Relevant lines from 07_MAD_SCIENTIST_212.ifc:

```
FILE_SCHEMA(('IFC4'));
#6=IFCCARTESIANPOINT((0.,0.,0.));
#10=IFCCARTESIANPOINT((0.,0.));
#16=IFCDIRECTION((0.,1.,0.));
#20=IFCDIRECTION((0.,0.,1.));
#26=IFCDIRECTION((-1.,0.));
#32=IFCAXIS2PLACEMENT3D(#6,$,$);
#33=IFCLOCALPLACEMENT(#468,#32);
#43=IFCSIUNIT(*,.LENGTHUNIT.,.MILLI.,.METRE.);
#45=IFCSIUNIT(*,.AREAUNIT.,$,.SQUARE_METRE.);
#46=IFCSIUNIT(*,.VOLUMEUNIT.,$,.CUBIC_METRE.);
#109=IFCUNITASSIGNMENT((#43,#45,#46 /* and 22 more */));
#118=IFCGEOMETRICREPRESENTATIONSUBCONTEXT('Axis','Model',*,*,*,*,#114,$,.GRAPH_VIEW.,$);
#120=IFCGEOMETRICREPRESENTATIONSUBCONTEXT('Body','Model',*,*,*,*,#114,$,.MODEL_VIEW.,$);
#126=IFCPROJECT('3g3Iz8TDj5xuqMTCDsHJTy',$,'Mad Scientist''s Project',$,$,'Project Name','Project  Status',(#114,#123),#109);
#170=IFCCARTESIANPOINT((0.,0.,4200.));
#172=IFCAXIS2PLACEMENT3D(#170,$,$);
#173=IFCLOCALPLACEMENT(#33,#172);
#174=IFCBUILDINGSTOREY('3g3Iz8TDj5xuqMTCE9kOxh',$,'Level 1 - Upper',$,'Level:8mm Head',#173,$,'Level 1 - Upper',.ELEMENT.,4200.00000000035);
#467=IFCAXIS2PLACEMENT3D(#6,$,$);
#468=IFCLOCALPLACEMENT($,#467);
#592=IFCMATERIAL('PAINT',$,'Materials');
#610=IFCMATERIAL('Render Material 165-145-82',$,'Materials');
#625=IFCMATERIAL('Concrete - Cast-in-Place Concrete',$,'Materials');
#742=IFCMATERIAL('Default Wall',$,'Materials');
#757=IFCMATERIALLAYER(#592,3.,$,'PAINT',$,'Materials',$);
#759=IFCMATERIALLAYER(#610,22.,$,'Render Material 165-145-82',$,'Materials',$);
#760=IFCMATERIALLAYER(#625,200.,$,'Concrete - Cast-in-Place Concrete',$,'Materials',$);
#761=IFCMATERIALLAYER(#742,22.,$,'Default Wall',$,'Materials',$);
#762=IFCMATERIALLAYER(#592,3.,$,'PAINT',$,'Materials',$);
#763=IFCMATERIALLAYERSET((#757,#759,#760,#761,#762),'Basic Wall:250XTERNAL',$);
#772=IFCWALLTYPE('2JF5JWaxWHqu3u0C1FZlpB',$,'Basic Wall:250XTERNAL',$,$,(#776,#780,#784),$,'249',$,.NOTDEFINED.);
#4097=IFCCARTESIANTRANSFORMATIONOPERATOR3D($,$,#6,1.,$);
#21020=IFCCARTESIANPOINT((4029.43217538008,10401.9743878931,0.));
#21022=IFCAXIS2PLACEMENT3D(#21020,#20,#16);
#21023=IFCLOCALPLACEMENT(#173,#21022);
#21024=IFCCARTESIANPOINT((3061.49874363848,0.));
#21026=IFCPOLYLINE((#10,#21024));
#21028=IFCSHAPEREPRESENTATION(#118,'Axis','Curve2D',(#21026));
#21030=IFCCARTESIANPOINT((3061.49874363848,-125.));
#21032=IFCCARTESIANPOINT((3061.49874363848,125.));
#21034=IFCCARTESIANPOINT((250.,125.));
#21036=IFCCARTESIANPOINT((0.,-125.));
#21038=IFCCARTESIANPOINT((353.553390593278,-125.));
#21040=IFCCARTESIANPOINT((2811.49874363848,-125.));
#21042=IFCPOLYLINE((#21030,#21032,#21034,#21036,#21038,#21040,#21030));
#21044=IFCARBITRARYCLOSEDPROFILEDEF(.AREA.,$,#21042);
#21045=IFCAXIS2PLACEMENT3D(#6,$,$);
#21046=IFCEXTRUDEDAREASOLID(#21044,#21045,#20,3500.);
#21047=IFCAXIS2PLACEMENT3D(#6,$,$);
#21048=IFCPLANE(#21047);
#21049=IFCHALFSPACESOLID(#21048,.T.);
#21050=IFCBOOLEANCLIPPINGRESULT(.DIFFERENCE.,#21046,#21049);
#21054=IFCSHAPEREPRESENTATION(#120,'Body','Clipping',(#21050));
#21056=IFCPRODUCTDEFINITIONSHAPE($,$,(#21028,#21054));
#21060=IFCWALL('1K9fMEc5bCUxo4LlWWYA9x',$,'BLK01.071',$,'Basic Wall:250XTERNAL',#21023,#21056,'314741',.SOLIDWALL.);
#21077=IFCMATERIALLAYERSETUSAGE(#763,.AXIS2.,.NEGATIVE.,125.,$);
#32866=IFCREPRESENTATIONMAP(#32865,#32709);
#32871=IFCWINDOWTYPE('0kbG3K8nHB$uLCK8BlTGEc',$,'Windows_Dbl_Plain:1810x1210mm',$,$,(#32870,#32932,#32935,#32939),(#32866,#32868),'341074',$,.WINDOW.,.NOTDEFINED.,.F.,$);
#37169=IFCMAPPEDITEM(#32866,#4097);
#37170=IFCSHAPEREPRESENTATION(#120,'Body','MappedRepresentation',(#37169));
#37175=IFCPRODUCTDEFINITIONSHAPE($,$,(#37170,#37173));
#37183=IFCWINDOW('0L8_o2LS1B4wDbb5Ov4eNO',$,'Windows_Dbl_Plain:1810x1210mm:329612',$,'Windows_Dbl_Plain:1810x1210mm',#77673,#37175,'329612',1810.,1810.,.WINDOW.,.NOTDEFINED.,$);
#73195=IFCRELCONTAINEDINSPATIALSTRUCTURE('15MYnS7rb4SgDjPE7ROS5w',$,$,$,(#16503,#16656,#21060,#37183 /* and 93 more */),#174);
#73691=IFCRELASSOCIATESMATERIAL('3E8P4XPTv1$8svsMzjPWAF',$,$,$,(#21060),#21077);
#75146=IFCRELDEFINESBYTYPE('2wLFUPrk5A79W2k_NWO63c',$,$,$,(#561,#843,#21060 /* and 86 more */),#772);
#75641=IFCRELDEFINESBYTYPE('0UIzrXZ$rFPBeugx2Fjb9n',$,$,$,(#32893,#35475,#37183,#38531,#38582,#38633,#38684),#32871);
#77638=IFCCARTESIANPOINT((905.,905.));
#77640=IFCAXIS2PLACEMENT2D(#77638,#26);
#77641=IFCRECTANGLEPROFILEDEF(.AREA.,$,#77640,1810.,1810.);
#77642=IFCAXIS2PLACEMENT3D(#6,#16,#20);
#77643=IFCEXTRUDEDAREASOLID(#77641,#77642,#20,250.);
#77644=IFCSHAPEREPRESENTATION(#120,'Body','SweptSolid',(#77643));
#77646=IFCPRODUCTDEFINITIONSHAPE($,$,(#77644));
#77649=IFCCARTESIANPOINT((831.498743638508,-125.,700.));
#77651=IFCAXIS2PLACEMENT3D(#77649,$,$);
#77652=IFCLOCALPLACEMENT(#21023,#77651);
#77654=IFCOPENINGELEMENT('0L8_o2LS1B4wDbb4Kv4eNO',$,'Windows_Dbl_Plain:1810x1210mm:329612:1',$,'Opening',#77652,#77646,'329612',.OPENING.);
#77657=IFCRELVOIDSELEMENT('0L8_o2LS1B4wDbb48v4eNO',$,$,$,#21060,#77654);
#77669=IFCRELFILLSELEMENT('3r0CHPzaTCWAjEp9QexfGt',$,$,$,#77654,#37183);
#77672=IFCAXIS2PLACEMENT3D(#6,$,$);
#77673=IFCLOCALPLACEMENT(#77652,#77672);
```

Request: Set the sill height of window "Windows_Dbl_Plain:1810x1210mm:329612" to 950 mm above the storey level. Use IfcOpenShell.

```python
import numpy as np
import ifcopenshell
import ifcopenshell.api.geometry
import ifcopenshell.geom
import ifcopenshell.util.element
import ifcopenshell.util.placement
import ifcopenshell.util.shape
import ifcopenshell.util.unit

model = ifcopenshell.open("07_MAD_SCIENTIST_212.ifc")
unit_scale = ifcopenshell.util.unit.calculate_unit_scale(model)

window = model.by_id(37183)
opening = window.FillsVoids[0].RelatingOpeningElement
storey = ifcopenshell.util.element.get_container(window, ifc_class="IfcBuildingStorey")
level = ifcopenshell.util.placement.get_local_placement(storey.ObjectPlacement)[2, 3]

# The opening's origin need not be at the sill, so measure its lowest point.
shape = ifcopenshell.geom.create_shape(ifcopenshell.geom.settings(), opening)
bottom = ifcopenshell.util.shape.get_shape_bottom_elevation(shape, shape.geometry) / unit_scale
dz = level + 950.0 - bottom

shift = np.array([0.0, 0.0, dz])
# The window is placed relative to its opening, so it follows when the opening moves.
matrix = ifcopenshell.util.placement.get_local_placement(opening.ObjectPlacement)
matrix[:3, 3] += shift
ifcopenshell.api.geometry.edit_object_placement(
    model, product=opening, matrix=matrix, is_si=False, should_transform_children=True
)

print(f"moved by {dz * unit_scale:+.3f} m")

model.write("07_MAD_SCIENTIST_212_v2.ifc")
```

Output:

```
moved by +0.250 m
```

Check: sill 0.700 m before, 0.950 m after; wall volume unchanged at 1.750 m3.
